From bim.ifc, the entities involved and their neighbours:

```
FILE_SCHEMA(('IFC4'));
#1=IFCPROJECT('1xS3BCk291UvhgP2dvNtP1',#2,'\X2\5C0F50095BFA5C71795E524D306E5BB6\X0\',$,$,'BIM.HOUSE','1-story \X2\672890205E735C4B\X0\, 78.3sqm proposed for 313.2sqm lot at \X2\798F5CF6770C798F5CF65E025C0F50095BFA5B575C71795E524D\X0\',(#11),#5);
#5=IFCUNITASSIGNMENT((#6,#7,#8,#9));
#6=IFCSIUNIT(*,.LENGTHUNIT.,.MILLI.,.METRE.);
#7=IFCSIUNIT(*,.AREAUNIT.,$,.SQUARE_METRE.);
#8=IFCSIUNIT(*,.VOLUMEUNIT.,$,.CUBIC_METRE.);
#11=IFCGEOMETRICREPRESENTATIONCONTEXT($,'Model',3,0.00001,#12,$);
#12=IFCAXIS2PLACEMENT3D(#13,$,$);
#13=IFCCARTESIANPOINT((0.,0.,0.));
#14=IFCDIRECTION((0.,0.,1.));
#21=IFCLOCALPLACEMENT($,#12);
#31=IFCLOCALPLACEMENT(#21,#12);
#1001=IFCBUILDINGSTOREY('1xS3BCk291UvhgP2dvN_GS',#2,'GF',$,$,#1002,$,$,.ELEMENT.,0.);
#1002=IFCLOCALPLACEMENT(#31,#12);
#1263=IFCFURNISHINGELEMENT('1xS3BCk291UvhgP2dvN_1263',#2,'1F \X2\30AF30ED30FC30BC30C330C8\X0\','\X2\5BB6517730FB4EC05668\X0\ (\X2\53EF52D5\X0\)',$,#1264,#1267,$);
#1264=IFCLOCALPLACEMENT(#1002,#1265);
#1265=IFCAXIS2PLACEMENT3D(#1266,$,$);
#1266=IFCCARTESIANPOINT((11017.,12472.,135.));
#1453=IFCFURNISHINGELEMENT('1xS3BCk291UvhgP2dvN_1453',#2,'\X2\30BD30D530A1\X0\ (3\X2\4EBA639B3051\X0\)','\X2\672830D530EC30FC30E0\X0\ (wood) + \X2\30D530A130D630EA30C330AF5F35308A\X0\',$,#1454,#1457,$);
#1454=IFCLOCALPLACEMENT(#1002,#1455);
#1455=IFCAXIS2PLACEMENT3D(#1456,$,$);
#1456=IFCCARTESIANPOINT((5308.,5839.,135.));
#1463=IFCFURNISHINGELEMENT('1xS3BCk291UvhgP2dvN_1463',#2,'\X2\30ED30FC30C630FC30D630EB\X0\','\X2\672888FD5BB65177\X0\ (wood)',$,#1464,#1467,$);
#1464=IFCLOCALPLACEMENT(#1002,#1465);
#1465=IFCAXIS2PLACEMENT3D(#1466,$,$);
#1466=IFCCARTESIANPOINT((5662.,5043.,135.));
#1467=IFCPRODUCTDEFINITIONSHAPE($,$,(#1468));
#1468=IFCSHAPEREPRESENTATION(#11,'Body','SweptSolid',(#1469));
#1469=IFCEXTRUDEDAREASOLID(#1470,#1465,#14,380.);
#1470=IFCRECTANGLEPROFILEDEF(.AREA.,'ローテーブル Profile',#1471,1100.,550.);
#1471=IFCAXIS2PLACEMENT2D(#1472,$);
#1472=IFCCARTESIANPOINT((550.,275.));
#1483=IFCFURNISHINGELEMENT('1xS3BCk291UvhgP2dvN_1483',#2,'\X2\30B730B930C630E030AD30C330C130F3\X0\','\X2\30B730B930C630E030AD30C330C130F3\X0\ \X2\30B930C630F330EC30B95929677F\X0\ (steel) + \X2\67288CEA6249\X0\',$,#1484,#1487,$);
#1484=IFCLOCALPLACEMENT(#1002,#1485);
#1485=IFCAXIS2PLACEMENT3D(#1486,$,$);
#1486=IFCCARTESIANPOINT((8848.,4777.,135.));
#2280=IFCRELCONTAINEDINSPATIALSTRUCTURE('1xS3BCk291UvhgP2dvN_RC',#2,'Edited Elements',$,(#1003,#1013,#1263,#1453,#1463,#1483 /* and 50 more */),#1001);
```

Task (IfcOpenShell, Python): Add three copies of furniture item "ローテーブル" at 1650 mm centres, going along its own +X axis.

```python
import ifcopenshell
import ifcopenshell.api.geometry
import ifcopenshell.api.root
import ifcopenshell.util.element
import ifcopenshell.util.placement

model = ifcopenshell.open("bim.ifc")


def reuse_history(source, copy):
    """copy_class also copies each property set's owner history, people and application; keep the originals."""
    for rel in copy.IsDefinedBy:
        if rel.is_a("IfcRelDefinesByProperties") and (history := rel.RelatingPropertyDefinition.OwnerHistory):
            rel.RelatingPropertyDefinition.OwnerHistory = source.OwnerHistory
            ifcopenshell.util.element.remove_deep2(model, history)


source = model.by_id(1463)
base = ifcopenshell.util.placement.get_local_placement(source.ObjectPlacement)
step = base[:3, 0] * 1650.0

for i in range(1, 4):
    copy = ifcopenshell.api.root.copy_class(model, product=source)
    copy.Representation = ifcopenshell.util.element.copy_deep(
        model, source.Representation, exclude=["IfcGeometricRepresentationContext", "IfcRepresentationMap"]
    )
    reuse_history(source, copy)
    matrix = base.copy()
    matrix[:3, 3] += i * step
    print("added at", matrix[:3, 3].round(3) + 0.0)
    ifcopenshell.api.geometry.edit_object_placement(model, product=copy, matrix=matrix, is_si=False)

model.write("bim_rev.ifc")
```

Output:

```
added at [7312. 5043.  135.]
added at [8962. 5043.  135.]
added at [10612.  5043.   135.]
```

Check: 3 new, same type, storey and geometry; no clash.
